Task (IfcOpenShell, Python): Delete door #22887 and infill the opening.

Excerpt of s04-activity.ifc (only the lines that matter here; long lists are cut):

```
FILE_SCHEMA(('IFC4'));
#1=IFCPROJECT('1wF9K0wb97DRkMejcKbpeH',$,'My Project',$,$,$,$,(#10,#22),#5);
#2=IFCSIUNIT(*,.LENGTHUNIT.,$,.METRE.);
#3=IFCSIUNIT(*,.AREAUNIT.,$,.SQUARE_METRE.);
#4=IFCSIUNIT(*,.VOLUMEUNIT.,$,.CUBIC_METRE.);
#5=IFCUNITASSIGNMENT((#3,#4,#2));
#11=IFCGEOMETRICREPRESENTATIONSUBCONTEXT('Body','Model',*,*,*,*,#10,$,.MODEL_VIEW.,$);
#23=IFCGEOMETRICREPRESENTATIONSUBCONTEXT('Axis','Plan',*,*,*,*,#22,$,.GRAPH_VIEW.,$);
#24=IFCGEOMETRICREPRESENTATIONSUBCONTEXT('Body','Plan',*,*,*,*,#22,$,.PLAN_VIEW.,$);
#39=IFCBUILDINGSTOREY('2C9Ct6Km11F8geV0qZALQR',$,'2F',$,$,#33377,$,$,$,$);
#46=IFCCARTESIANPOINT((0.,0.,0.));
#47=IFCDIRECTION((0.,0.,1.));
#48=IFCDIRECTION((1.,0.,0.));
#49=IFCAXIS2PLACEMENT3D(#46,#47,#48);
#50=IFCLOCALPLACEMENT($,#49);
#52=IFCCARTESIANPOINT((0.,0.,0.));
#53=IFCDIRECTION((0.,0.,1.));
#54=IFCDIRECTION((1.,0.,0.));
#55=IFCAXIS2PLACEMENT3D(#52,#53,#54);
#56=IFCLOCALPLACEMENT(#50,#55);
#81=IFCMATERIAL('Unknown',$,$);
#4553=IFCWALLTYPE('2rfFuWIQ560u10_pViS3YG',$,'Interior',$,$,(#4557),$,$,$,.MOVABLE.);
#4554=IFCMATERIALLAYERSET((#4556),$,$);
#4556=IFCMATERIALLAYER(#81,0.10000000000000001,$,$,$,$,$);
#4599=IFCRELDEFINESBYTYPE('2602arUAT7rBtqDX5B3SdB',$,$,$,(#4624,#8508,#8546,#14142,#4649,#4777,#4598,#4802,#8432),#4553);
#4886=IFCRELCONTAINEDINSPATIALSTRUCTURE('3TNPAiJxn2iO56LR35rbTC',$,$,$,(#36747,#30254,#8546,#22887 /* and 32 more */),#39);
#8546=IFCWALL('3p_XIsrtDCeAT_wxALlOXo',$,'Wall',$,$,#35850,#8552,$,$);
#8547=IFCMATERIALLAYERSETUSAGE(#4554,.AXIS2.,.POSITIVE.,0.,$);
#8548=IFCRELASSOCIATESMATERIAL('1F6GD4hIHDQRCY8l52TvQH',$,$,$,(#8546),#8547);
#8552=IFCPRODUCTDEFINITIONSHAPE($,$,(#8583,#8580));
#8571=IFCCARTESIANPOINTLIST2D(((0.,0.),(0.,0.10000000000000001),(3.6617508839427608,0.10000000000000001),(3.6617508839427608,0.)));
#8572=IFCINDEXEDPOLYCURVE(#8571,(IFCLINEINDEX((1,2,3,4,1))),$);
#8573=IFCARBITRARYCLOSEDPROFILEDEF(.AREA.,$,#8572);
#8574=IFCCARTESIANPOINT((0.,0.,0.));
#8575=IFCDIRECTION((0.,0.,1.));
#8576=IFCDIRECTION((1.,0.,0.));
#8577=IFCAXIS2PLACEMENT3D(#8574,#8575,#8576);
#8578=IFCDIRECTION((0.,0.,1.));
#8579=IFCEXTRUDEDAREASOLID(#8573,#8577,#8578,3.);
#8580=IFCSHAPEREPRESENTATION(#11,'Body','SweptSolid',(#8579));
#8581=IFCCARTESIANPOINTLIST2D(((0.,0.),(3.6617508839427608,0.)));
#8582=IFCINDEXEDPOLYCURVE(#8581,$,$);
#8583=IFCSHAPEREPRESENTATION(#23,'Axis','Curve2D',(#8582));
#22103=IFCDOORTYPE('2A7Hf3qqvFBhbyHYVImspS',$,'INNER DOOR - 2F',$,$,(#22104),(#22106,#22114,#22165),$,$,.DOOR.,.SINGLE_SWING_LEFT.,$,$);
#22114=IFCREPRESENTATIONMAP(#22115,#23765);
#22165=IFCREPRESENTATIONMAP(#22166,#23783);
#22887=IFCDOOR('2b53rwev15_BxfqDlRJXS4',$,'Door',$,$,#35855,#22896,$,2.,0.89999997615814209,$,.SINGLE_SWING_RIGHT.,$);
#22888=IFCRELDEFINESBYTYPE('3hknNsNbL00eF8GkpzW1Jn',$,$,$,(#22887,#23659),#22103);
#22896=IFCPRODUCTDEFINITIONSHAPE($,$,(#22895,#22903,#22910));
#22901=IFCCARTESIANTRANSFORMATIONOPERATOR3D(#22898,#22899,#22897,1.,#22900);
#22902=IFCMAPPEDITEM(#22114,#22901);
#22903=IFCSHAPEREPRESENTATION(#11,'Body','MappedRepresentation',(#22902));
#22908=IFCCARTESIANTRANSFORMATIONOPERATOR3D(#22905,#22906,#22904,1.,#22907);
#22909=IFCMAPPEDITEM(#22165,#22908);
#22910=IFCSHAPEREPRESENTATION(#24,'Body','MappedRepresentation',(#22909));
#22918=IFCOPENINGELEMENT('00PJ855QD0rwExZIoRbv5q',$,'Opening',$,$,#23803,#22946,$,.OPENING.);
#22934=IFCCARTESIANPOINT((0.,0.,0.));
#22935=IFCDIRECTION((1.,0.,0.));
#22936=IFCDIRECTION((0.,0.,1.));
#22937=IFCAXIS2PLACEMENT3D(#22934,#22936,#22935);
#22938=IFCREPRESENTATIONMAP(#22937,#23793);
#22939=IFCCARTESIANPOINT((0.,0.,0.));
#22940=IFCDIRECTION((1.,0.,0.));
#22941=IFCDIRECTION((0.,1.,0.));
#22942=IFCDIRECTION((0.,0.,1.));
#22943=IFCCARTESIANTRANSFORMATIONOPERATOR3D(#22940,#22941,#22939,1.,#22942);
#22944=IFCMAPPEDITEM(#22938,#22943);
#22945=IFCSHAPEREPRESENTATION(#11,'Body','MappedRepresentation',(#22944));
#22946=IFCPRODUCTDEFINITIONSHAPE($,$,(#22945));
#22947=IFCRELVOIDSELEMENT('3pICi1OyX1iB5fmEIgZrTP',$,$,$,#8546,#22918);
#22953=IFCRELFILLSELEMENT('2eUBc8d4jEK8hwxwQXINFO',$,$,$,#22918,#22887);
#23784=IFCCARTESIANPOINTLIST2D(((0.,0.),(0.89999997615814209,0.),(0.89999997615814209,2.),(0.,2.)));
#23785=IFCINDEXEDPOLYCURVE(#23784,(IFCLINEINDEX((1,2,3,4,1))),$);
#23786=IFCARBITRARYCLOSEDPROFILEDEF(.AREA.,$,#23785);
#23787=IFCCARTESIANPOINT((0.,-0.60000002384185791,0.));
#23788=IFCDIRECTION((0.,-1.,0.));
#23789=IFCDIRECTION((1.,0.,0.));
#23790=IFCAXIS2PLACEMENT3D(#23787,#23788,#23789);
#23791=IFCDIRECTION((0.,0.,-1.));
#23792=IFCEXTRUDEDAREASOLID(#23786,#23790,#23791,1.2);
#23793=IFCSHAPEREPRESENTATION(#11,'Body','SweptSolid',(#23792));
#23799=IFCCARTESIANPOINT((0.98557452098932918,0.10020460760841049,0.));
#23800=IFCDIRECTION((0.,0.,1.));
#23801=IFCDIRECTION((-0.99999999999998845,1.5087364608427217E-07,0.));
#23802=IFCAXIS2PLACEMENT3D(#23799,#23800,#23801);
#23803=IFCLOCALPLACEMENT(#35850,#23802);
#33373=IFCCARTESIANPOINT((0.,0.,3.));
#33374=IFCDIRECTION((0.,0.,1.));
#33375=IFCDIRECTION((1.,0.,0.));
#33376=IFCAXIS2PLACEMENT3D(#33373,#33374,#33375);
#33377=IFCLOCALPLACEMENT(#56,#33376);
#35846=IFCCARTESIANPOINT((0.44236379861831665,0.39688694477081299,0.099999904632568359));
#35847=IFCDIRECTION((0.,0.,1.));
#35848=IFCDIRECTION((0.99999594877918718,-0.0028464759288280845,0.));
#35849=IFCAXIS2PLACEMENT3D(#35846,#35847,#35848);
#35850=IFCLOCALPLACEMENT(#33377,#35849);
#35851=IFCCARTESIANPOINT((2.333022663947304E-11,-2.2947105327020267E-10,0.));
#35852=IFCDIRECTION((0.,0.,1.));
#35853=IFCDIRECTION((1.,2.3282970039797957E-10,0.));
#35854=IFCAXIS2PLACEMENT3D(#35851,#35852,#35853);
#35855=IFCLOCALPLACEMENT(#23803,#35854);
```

```python
import ifcopenshell
import ifcopenshell.api.feature
import ifcopenshell.api.root
import ifcopenshell.geom
import ifcopenshell.util.shape

model = ifcopenshell.open("s04-activity.ifc")
settings = ifcopenshell.geom.settings()


def volume(element):
    """Net volume in cubic metres, openings subtracted."""
    shape = ifcopenshell.geom.create_shape(settings, element)
    return ifcopenshell.util.shape.get_volume(shape.geometry)


door = model.by_guid("2b53rwev15_BxfqDlRJXS4")
opening = door.FillsVoids[0].RelatingOpeningElement
wall = opening.VoidsElements[0].RelatingBuildingElement
before = volume(wall)

ifcopenshell.api.root.remove_product(model, product=door)
ifcopenshell.api.feature.remove_feature(model, feature=opening)

after = volume(wall)

print(f"wall volume {before:.3f} -> {after:.3f} m3")

model.write("s04-activity_v2.ifc")
```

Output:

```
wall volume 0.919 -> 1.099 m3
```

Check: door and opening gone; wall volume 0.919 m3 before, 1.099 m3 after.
